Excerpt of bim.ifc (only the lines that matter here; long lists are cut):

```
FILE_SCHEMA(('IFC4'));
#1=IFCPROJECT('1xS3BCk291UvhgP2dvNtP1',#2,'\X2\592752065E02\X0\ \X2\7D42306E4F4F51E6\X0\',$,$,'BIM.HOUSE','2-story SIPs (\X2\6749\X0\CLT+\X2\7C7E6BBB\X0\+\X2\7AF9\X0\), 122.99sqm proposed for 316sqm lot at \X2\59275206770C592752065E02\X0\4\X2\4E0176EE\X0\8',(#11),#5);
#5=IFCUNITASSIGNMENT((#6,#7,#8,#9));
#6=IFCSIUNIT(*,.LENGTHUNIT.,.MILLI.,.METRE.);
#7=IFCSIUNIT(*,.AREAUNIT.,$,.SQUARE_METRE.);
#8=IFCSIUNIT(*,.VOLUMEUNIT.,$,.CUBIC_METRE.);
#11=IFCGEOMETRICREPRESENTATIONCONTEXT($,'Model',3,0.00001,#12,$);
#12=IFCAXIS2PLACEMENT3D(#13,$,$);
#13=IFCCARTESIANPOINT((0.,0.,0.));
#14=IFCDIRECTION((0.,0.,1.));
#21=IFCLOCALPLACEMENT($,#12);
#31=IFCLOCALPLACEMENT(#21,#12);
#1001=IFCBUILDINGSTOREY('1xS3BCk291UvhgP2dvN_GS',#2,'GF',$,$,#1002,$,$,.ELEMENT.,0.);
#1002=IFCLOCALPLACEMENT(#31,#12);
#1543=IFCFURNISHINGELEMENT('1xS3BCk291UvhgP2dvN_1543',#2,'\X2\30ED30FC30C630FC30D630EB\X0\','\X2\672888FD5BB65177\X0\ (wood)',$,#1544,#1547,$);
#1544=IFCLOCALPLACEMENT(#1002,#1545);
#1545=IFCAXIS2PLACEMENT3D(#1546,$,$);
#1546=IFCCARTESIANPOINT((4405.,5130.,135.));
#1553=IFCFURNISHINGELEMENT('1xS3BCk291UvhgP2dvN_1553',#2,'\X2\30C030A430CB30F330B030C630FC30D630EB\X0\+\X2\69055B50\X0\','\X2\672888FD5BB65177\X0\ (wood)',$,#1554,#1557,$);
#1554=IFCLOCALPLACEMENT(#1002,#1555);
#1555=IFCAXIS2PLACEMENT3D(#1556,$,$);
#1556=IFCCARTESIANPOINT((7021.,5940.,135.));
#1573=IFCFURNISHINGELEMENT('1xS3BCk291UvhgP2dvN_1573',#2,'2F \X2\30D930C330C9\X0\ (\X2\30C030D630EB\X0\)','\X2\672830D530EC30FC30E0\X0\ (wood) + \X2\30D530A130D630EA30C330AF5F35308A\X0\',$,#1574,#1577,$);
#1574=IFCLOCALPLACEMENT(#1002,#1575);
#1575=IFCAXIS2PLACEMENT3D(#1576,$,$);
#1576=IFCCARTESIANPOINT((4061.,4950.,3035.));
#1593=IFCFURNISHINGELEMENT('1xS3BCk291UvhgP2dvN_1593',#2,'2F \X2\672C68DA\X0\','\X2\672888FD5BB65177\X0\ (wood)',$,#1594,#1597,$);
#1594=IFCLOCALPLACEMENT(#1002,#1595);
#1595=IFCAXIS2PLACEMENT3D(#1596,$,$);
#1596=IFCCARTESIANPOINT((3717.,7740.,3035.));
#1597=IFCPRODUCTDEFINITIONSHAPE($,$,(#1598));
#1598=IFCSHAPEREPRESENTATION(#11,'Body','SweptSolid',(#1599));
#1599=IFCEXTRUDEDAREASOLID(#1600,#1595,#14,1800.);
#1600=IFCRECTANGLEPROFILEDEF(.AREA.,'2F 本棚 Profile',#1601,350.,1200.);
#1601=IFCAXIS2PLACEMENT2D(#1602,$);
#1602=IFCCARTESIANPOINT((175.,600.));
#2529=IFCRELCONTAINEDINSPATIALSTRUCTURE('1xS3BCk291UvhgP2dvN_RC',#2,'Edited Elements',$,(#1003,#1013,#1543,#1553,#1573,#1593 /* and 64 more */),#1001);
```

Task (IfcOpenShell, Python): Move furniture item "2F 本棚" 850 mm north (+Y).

```python
import ifcopenshell
import ifcopenshell.api.geometry
import ifcopenshell.util.placement

model = ifcopenshell.open("bim.ifc")

item = model.by_guid("1xS3BCk291UvhgP2dvN_1593")
matrix = ifcopenshell.util.placement.get_local_placement(item.ObjectPlacement)
matrix[1, 3] += 850.0
ifcopenshell.api.geometry.edit_object_placement(model, product=item, matrix=matrix, is_si=False)

print(ifcopenshell.util.placement.get_local_placement(item.ObjectPlacement).round(3) + 0.0)

model.write("bim_rev.ifc")
```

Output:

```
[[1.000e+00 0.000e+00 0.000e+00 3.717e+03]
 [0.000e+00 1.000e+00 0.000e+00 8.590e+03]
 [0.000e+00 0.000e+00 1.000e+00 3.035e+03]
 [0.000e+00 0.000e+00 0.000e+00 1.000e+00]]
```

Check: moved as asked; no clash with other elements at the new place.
